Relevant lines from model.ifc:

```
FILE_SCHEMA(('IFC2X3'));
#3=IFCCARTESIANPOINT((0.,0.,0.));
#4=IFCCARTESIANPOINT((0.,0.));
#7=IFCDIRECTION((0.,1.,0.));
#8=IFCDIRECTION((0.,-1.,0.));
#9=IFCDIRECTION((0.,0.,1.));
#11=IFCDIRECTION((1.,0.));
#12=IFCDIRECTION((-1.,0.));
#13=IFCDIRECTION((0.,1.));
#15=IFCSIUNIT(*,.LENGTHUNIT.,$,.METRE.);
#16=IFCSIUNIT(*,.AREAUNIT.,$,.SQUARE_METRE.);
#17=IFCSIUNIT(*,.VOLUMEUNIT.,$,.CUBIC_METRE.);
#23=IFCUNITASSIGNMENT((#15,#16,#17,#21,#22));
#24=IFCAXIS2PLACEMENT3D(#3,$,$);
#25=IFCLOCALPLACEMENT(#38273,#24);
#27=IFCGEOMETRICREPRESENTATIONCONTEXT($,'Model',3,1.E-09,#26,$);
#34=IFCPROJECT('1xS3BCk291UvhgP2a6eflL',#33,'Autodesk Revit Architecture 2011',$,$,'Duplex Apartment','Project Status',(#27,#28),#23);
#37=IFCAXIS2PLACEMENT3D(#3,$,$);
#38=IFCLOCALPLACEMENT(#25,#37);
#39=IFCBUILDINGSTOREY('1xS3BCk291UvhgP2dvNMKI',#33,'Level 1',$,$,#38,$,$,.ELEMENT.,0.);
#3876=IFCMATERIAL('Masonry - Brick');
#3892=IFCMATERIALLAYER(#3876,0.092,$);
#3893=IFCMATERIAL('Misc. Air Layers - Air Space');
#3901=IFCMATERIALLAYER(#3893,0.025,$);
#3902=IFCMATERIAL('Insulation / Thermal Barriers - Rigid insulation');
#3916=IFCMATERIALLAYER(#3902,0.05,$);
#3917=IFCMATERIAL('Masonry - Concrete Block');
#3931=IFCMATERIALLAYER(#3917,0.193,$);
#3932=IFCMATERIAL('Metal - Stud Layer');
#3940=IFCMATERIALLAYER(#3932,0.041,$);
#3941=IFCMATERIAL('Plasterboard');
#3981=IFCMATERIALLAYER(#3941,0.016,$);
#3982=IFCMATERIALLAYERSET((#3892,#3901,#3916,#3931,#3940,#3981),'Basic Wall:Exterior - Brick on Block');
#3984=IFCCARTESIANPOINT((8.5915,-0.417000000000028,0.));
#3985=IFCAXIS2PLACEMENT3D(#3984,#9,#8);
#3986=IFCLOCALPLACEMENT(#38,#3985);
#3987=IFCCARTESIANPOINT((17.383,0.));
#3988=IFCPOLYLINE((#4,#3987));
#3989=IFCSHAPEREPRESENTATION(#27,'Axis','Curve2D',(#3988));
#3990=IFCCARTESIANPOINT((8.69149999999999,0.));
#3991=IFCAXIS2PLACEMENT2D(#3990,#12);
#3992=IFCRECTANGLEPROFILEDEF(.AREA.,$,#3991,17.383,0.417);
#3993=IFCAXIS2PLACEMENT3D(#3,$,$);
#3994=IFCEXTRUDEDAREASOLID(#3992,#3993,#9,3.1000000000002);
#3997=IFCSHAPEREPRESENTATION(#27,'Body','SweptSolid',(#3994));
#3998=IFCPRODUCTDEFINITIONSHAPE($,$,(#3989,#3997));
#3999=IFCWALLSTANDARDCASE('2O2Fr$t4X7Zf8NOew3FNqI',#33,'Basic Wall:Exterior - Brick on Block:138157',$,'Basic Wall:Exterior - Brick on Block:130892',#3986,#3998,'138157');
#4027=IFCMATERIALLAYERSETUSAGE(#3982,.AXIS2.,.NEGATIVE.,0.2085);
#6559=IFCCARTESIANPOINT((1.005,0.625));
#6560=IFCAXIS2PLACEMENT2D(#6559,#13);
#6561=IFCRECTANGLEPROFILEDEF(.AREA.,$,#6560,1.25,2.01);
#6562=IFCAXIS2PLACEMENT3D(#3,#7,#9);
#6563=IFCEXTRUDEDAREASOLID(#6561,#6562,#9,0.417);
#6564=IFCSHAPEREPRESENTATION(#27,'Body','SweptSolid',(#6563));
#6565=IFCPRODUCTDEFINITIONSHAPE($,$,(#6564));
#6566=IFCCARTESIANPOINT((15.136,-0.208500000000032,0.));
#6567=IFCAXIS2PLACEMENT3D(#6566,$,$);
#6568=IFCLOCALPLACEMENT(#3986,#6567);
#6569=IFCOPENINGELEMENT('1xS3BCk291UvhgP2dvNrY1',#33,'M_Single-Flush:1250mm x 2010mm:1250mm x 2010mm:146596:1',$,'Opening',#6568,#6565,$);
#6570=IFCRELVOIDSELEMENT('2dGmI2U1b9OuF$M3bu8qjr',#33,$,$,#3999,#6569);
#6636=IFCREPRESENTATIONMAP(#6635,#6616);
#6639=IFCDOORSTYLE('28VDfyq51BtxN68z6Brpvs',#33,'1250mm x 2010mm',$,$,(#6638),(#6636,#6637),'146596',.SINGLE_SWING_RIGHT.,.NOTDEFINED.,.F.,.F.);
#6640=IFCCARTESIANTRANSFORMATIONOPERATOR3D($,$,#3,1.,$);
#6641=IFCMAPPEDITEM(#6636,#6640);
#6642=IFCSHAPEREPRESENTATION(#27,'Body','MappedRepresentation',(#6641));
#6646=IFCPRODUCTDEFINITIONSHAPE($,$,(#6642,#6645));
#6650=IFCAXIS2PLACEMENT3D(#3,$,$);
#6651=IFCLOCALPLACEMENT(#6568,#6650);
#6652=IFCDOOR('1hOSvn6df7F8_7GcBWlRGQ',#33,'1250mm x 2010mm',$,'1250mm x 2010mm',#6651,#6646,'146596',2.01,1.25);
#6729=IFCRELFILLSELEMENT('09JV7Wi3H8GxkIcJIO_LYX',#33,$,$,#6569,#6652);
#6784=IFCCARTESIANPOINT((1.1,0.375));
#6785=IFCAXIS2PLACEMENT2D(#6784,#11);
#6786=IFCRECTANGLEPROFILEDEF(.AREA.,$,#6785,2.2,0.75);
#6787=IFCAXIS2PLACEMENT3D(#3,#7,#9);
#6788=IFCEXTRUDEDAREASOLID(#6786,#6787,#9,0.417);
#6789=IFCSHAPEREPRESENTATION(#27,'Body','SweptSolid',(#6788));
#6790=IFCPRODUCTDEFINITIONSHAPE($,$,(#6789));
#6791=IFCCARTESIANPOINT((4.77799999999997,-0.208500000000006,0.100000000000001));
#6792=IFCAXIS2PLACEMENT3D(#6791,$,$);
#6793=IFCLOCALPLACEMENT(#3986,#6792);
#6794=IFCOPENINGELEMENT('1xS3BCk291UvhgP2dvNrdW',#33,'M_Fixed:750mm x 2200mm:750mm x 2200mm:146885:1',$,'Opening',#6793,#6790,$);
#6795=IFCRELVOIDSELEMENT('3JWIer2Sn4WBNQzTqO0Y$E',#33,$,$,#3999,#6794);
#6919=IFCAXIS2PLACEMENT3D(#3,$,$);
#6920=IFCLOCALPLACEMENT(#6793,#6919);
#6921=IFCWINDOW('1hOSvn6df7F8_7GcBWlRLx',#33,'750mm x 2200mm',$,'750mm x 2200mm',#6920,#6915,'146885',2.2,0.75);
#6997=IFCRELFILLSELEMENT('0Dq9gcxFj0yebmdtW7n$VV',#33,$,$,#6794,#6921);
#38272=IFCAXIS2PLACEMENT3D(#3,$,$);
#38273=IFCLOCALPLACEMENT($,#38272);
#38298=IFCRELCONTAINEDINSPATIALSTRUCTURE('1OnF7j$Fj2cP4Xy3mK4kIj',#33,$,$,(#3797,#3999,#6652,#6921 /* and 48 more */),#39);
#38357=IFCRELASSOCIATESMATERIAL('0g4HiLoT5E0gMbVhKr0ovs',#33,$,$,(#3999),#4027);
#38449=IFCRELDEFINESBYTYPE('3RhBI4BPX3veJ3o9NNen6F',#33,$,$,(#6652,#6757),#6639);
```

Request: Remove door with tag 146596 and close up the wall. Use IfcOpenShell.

```python
import ifcopenshell
import ifcopenshell.api.feature
import ifcopenshell.api.root
import ifcopenshell.geom
import ifcopenshell.util.shape

model = ifcopenshell.open("model.ifc")
settings = ifcopenshell.geom.settings()


def volume(element):
    """Net volume in cubic metres, openings subtracted."""
    shape = ifcopenshell.geom.create_shape(settings, element)
    return ifcopenshell.util.shape.get_volume(shape.geometry)


door = model.by_guid("1hOSvn6df7F8_7GcBWlRGQ")
opening = door.FillsVoids[0].RelatingOpeningElement
wall = opening.VoidsElements[0].RelatingBuildingElement
before = volume(wall)

ifcopenshell.api.root.remove_product(model, product=door)
ifcopenshell.api.feature.remove_feature(model, feature=opening)

after = volume(wall)

print(f"wall volume {before:.3f} -> {after:.3f} m3")

model.write("model_v2.ifc")
```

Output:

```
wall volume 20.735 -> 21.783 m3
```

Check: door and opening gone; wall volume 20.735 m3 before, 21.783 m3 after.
